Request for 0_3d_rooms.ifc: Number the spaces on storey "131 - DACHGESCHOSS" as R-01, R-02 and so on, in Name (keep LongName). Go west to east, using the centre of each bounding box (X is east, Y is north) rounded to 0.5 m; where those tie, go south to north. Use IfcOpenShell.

First a look at what the model holds.

```python
import ifcopenshell
import ifcopenshell.util.element
import ifcopenshell.util.placement

model = ifcopenshell.open("0_3d_rooms.ifc")
print(model.schema)
storey = next(s for s in model.by_type("IfcBuildingStorey") if s.Name == "131 - DACHGESCHOSS")
spaces = [e for e in ifcopenshell.util.element.get_decomposition(storey) if e.is_a("IfcSpace")]
for e in sorted(spaces, key=lambda e: e.id()):
    origin = ifcopenshell.util.placement.get_local_placement(e.ObjectPlacement)[:3, 3]
    print(e.id(), e.Name, e.LongName, origin.round(2) + 0.0, sep=" | ")
```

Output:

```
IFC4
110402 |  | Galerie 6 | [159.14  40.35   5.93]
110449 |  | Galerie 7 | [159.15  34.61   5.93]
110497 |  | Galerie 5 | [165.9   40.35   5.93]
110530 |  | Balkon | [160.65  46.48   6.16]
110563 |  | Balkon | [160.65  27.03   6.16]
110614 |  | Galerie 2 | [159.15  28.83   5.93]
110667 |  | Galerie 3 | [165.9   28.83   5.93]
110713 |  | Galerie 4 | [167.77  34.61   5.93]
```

```python
import ifcopenshell
import ifcopenshell.geom
import ifcopenshell.util.element
import ifcopenshell.util.shape

model = ifcopenshell.open("0_3d_rooms.ifc")
settings = ifcopenshell.geom.settings()
settings.set("use-world-coords", True)


def centre(element):
    shape = ifcopenshell.geom.create_shape(settings, element)
    return ifcopenshell.util.shape.get_bbox_centroid(shape.geometry)


storey = next(s for s in model.by_type("IfcBuildingStorey") if s.Name == "131 - DACHGESCHOSS")
spaces = [e for e in ifcopenshell.util.element.get_decomposition(storey) if e.is_a("IfcSpace")]

# Insertion points can sit at a corner or the storey origin, so sort by the geometry (in metres).
centres = {e: centre(e) for e in spaces}
spaces.sort(key=lambda e: (round(centres[e][0] / 0.5), centres[e][1]))

for i, e in enumerate(spaces, start=1):
    number = f"R-{i:02d}"
    e.Name = number
    print(e.id(), number)

model.write("0_3d_rooms_edited.ifc")
```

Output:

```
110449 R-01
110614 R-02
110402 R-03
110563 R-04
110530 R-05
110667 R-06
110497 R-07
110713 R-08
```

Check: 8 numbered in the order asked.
